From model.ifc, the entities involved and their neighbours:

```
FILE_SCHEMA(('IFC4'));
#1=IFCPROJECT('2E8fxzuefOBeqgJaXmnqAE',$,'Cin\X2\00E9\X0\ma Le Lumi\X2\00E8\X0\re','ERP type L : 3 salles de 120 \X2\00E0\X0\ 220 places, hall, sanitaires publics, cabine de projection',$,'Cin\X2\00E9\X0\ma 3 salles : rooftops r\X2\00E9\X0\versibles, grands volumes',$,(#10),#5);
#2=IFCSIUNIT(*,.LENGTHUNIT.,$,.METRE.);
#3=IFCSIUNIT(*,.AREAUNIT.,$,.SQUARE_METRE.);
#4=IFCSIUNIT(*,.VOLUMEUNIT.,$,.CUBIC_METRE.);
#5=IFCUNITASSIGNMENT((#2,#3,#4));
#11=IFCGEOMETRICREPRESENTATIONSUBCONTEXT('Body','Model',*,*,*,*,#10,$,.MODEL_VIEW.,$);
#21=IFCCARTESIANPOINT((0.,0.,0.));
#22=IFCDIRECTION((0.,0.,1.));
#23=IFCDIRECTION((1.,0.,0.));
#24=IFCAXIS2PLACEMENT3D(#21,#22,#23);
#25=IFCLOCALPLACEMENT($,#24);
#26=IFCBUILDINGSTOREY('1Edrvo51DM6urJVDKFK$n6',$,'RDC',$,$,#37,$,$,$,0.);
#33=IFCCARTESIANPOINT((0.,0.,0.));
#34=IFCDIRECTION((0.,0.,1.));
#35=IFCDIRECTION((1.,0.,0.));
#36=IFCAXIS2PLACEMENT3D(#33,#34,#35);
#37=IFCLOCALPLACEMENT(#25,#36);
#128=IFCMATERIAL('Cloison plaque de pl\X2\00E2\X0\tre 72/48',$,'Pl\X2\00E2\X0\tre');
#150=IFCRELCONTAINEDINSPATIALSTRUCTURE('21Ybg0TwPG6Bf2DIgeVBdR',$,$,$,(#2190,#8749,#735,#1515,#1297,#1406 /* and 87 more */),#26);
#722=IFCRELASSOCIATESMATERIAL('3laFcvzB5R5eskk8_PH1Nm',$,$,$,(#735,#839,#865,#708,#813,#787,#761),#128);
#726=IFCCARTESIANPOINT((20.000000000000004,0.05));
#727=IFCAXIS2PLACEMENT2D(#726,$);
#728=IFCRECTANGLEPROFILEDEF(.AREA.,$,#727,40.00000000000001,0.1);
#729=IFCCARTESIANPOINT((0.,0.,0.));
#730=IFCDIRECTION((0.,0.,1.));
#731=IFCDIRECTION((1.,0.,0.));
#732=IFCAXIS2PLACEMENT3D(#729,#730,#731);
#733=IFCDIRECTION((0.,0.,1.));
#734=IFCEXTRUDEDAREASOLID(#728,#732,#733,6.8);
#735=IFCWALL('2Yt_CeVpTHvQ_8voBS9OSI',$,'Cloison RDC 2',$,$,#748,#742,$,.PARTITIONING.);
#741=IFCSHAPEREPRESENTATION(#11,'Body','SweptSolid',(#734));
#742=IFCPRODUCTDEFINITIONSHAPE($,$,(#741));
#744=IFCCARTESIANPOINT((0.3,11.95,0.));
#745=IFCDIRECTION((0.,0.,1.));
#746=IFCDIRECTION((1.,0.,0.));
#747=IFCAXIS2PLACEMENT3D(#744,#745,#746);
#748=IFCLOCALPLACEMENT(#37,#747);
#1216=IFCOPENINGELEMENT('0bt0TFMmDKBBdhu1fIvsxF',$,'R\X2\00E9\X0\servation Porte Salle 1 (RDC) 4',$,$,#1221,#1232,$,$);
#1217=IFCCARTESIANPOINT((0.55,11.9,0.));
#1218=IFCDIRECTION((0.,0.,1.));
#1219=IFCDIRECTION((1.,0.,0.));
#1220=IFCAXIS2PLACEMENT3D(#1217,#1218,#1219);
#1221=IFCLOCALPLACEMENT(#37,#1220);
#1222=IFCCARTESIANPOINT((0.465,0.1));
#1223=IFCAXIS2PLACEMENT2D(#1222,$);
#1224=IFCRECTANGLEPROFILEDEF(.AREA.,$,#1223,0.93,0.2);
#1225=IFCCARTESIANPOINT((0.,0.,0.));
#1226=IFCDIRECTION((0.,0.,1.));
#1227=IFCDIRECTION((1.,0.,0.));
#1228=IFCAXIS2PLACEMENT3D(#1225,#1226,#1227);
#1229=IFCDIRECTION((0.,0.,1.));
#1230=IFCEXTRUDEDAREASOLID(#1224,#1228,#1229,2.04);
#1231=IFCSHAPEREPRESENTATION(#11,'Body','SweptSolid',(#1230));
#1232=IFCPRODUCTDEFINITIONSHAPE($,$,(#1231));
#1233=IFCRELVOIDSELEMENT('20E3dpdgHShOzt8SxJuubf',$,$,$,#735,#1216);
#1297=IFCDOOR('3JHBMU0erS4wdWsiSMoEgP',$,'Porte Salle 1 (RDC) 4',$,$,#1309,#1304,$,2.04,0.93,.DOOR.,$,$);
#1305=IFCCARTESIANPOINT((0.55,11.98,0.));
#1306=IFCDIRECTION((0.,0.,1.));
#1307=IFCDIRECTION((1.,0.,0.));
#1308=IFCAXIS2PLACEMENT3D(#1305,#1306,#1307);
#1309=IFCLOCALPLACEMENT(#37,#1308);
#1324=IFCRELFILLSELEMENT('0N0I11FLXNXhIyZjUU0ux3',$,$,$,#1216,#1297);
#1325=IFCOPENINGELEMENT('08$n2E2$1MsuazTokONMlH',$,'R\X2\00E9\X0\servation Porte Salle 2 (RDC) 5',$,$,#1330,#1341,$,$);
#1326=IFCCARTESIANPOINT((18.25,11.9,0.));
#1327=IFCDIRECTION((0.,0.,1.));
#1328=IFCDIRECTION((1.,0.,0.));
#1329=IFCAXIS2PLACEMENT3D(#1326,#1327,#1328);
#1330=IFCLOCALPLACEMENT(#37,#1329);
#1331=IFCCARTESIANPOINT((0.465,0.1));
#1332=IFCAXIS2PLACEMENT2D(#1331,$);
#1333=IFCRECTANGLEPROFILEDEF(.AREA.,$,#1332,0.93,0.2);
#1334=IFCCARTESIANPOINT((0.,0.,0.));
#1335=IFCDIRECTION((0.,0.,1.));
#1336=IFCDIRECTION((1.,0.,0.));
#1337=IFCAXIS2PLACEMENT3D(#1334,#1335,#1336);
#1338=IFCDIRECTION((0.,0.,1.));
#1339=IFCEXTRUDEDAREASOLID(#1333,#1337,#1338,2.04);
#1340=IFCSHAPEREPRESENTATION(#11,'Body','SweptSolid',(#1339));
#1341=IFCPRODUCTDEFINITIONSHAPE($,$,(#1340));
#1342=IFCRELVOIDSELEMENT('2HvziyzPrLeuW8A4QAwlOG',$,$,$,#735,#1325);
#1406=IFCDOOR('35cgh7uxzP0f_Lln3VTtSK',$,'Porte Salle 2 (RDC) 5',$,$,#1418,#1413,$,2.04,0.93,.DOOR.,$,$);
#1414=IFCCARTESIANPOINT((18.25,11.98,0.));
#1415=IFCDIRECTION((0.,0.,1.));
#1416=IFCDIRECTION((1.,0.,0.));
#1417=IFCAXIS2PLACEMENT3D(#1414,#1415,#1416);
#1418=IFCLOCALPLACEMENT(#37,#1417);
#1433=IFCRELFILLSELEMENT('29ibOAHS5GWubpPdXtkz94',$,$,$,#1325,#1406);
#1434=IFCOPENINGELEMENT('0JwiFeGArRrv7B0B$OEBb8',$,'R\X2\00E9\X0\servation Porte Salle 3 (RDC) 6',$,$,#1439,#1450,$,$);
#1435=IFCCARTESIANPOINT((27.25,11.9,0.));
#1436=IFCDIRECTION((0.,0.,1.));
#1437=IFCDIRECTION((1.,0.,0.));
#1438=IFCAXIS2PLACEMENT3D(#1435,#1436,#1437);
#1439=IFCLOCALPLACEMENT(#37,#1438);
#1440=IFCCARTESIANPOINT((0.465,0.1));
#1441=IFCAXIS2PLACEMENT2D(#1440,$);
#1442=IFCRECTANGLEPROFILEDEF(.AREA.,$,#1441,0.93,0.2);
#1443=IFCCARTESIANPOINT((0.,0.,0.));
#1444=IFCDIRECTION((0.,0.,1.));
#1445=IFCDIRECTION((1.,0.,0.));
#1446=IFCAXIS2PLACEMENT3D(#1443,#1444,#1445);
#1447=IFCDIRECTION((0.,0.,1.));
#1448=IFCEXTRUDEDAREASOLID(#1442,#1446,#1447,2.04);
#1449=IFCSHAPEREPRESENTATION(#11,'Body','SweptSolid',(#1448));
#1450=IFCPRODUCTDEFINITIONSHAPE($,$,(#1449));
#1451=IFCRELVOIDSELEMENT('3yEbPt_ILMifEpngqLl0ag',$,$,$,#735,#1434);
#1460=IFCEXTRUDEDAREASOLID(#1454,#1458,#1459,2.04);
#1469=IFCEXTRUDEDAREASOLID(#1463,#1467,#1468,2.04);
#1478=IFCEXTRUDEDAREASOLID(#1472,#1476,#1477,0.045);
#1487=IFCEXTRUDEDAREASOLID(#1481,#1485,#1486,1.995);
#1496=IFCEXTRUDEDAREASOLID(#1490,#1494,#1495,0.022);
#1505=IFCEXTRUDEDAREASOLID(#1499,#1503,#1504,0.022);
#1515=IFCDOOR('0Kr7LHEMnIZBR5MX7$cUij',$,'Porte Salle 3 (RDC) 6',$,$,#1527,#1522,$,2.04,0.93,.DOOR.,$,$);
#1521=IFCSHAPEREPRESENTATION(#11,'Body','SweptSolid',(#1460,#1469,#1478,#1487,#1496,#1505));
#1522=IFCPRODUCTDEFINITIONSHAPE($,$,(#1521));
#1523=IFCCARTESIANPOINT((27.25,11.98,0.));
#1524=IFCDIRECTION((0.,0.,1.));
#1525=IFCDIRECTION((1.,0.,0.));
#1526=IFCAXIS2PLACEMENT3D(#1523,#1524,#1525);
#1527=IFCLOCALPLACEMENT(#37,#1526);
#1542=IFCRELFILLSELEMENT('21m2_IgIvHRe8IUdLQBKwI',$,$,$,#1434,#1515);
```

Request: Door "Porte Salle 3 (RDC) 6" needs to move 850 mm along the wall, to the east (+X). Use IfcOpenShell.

```python
import ifcopenshell
import ifcopenshell.api.geometry
import ifcopenshell.util.placement
import ifcopenshell.util.unit

model = ifcopenshell.open("model.ifc")
unit_scale = ifcopenshell.util.unit.calculate_unit_scale(model)

door = model.by_id(1515)
opening = door.FillsVoids[0].RelatingOpeningElement
wall = opening.VoidsElements[0].RelatingBuildingElement

wall_matrix = ifcopenshell.util.placement.get_local_placement(wall.ObjectPlacement)
shift = wall_matrix[:3, 0] * 0.85 / unit_scale
before = ifcopenshell.util.placement.get_local_placement(door.ObjectPlacement)[:3, 3].copy()

# The door is not placed relative to its opening, so move both.
for product in (opening, door):
    matrix = ifcopenshell.util.placement.get_local_placement(product.ObjectPlacement)
    matrix[:3, 3] += shift
    ifcopenshell.api.geometry.edit_object_placement(model, product=product, matrix=matrix, is_si=False)

after = ifcopenshell.util.placement.get_local_placement(door.ObjectPlacement)[:3, 3]
print("door moved by", (after - before).round(3) + 0.0)

model.write("model_updated.ifc")
```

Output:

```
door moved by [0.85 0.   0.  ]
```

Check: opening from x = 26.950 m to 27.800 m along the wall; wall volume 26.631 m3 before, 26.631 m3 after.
